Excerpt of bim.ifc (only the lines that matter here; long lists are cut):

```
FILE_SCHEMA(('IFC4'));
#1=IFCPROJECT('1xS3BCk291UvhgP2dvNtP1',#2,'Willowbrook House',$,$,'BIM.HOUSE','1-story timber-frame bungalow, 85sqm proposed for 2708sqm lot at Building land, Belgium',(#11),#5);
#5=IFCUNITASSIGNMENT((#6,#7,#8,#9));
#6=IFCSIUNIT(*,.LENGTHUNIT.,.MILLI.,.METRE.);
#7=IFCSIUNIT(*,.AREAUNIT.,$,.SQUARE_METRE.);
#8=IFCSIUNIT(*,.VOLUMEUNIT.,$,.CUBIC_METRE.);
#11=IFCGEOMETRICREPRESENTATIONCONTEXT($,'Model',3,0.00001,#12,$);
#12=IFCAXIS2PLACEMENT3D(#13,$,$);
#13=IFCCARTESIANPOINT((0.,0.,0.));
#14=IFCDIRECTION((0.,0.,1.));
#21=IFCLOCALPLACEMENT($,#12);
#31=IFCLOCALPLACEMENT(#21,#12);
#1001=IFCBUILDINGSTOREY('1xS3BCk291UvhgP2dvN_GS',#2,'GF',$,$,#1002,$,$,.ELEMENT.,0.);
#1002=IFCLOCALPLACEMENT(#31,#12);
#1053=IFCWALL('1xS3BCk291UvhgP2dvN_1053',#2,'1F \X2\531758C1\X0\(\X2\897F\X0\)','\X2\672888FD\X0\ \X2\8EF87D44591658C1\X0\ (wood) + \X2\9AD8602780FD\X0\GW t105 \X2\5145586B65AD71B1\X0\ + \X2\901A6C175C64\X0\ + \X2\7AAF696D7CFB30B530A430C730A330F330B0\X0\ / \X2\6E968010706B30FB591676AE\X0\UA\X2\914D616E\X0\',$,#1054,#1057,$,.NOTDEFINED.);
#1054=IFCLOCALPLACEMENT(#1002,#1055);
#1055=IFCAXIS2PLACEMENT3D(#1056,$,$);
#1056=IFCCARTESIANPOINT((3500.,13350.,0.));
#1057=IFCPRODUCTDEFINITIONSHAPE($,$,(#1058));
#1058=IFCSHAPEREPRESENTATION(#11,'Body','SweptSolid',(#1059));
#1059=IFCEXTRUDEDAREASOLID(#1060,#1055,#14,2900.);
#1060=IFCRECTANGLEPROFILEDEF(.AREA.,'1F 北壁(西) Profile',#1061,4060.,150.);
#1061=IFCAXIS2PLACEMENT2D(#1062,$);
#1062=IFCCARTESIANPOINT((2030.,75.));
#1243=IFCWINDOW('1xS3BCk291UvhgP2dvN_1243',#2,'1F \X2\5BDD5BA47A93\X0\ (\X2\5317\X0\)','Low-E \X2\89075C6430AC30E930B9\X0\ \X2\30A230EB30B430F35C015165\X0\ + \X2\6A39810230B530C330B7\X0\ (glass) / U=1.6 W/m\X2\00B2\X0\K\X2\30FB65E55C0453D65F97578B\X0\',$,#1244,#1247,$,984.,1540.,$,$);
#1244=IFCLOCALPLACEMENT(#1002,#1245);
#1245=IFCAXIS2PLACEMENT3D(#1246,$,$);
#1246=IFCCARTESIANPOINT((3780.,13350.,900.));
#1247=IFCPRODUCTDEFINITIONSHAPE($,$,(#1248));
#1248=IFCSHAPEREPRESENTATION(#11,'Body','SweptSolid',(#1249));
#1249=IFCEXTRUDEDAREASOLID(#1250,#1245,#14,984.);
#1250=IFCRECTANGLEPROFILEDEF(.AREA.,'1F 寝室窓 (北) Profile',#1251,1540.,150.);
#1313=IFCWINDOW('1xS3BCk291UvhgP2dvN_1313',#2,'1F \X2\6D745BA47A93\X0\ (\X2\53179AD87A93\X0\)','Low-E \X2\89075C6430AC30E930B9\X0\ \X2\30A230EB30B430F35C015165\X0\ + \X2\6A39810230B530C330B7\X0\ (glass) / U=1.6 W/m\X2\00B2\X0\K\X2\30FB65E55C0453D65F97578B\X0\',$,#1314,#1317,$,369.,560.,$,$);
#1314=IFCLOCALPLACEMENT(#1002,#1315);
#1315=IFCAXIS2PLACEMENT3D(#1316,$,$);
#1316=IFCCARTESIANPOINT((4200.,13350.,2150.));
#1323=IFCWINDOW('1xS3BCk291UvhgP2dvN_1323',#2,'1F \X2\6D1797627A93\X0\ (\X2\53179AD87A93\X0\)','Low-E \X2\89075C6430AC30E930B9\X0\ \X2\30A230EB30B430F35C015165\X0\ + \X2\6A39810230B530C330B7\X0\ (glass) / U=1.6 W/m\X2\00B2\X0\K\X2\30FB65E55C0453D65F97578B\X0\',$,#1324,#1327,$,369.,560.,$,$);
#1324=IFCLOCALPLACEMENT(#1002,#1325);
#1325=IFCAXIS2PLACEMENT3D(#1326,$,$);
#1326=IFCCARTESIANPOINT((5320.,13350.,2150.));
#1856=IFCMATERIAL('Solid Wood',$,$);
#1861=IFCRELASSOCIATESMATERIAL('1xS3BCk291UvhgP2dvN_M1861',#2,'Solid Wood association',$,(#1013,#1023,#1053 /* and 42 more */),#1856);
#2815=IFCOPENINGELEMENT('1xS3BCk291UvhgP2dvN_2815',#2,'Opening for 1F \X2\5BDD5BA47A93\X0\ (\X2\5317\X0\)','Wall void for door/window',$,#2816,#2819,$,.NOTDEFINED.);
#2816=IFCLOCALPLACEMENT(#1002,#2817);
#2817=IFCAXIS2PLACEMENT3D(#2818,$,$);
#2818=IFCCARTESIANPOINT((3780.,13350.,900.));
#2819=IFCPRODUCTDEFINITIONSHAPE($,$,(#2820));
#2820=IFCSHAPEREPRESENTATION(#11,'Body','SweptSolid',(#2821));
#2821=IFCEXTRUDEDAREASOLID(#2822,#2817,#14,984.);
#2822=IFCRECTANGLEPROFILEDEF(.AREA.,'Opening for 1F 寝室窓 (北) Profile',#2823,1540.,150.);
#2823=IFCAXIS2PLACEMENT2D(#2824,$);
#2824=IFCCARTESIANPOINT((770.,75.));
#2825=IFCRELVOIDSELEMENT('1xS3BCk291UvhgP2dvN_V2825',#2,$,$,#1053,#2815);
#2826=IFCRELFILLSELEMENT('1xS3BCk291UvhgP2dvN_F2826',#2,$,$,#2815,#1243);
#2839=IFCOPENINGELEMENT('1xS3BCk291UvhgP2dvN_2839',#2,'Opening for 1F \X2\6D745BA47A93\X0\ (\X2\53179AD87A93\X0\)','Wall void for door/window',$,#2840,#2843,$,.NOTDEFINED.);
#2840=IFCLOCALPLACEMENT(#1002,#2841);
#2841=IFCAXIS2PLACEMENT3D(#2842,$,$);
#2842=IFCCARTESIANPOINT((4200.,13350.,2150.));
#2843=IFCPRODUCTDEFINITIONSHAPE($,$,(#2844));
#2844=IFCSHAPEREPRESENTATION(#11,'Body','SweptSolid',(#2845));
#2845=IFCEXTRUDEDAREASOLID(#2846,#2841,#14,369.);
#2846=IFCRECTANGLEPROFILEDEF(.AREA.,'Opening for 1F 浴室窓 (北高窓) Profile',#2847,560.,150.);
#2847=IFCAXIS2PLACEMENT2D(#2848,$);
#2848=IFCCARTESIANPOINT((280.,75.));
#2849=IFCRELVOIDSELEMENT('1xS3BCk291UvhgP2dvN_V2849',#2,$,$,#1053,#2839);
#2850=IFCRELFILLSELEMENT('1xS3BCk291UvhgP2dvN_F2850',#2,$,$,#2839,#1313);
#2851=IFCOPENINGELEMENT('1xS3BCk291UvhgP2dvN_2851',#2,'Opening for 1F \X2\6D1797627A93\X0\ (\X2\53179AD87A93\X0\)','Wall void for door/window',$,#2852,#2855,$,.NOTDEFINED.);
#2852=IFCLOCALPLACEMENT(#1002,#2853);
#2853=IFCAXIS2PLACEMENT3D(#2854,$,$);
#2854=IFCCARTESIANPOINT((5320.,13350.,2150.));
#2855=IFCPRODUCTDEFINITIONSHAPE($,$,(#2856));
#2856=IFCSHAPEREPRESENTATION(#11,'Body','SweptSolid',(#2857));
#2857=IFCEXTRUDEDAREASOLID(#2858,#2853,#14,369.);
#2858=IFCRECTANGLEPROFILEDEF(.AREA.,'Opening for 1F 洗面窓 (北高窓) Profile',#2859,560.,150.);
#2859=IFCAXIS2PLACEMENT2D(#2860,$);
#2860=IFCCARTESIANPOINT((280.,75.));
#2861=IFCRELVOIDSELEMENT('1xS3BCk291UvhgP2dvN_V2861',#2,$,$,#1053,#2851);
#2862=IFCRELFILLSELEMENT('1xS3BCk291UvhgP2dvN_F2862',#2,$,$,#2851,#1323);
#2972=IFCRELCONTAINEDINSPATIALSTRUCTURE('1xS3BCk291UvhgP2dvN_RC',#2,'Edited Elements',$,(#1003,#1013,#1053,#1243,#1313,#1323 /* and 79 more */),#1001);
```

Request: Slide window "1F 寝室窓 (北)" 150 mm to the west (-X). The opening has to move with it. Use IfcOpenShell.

```python
import ifcopenshell
import ifcopenshell.api.geometry
import ifcopenshell.util.placement
import ifcopenshell.util.unit

model = ifcopenshell.open("bim.ifc")
unit_scale = ifcopenshell.util.unit.calculate_unit_scale(model)

window = model.by_guid("1xS3BCk291UvhgP2dvN_1243")
opening = window.FillsVoids[0].RelatingOpeningElement
wall = opening.VoidsElements[0].RelatingBuildingElement

wall_matrix = ifcopenshell.util.placement.get_local_placement(wall.ObjectPlacement)
shift = wall_matrix[:3, 0] * -0.15 / unit_scale
before = ifcopenshell.util.placement.get_local_placement(window.ObjectPlacement)[:3, 3].copy()

# The window is not placed relative to its opening, so move both.
for product in (opening, window):
    matrix = ifcopenshell.util.placement.get_local_placement(product.ObjectPlacement)
    matrix[:3, 3] += shift
    ifcopenshell.api.geometry.edit_object_placement(model, product=product, matrix=matrix, is_si=False)

after = ifcopenshell.util.placement.get_local_placement(window.ObjectPlacement)[:3, 3]
print("window moved by", (after - before).round(3) + 0.0)

model.write("bim_updated.ifc")
```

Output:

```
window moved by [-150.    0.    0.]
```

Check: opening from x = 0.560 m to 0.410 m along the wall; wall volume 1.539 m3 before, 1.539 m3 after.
